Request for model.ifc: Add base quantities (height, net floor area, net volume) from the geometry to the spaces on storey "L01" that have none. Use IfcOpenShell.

First a look at what the model holds.

```python
import ifcopenshell
import ifcopenshell.util.element
import ifcopenshell.util.unit

model = ifcopenshell.open("model.ifc")
print(model.schema)
for unit_type in ("LENGTHUNIT", "AREAUNIT", "VOLUMEUNIT"):
    print(unit_type, ifcopenshell.util.unit.calculate_unit_scale(model, unit_type))
storey = next(s for s in model.by_type("IfcBuildingStorey") if s.Name == "L01")
spaces = [e for e in ifcopenshell.util.element.get_decomposition(storey) if e.is_a("IfcSpace")]
for e in sorted(spaces, key=lambda e: e.id()):
    print(e.id(), e.is_a(), e.Name, list(ifcopenshell.util.element.get_psets(e, qtos_only=True)), sep=" | ")
```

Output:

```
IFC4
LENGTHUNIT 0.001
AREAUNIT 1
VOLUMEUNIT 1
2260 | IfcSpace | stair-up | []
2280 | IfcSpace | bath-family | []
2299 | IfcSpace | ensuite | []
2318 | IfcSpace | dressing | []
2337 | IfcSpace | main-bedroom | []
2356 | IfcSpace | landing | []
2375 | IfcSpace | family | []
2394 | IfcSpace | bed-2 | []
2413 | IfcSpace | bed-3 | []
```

```python
import ifcopenshell
import ifcopenshell.api.pset
import ifcopenshell.geom
import ifcopenshell.util.element
import ifcopenshell.util.shape
import ifcopenshell.util.unit

model = ifcopenshell.open("model.ifc")
unit_scale = ifcopenshell.util.unit.calculate_unit_scale(model)
area_scale = ifcopenshell.util.unit.calculate_unit_scale(model, "AREAUNIT")
volume_scale = ifcopenshell.util.unit.calculate_unit_scale(model, "VOLUMEUNIT")
settings = ifcopenshell.geom.settings()

storey = next(s for s in model.by_type("IfcBuildingStorey") if s.Name == "L01")
spaces = [e for e in ifcopenshell.util.element.get_decomposition(storey) if e.is_a("IfcSpace")]

for e in sorted(spaces, key=lambda e: e.id()):
    if ifcopenshell.util.element.get_psets(e, qtos_only=True, should_inherit=False):
        continue
    # Geometry comes back in metres, in the element's own axes.
    shape = ifcopenshell.geom.create_shape(settings, e)
    values = {
        "Height": ifcopenshell.util.shape.get_z(shape.geometry) / unit_scale,
        "NetFloorArea": ifcopenshell.util.shape.get_footprint_area(shape.geometry) / area_scale,
        "NetVolume": ifcopenshell.util.shape.get_volume(shape.geometry) / volume_scale,
    }
    qto = ifcopenshell.api.pset.add_qto(model, product=e, name="Qto_SpaceBaseQuantities")
    ifcopenshell.api.pset.edit_qto(model, qto=qto, properties=values)
    print(e.id(), {k: round(v, 3) for k, v in values.items()})

model.write("model_updated.ifc")
```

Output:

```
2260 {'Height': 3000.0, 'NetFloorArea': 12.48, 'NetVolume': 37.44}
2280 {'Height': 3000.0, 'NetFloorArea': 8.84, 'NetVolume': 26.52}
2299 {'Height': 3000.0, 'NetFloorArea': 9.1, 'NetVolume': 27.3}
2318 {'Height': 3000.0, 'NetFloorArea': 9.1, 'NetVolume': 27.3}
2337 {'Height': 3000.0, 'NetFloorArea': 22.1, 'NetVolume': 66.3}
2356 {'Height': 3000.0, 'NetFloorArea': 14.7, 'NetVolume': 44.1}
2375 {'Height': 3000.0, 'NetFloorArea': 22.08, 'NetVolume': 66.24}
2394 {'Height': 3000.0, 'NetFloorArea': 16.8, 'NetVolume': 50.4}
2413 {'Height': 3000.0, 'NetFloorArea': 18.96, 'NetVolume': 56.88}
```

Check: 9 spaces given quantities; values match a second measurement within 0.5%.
